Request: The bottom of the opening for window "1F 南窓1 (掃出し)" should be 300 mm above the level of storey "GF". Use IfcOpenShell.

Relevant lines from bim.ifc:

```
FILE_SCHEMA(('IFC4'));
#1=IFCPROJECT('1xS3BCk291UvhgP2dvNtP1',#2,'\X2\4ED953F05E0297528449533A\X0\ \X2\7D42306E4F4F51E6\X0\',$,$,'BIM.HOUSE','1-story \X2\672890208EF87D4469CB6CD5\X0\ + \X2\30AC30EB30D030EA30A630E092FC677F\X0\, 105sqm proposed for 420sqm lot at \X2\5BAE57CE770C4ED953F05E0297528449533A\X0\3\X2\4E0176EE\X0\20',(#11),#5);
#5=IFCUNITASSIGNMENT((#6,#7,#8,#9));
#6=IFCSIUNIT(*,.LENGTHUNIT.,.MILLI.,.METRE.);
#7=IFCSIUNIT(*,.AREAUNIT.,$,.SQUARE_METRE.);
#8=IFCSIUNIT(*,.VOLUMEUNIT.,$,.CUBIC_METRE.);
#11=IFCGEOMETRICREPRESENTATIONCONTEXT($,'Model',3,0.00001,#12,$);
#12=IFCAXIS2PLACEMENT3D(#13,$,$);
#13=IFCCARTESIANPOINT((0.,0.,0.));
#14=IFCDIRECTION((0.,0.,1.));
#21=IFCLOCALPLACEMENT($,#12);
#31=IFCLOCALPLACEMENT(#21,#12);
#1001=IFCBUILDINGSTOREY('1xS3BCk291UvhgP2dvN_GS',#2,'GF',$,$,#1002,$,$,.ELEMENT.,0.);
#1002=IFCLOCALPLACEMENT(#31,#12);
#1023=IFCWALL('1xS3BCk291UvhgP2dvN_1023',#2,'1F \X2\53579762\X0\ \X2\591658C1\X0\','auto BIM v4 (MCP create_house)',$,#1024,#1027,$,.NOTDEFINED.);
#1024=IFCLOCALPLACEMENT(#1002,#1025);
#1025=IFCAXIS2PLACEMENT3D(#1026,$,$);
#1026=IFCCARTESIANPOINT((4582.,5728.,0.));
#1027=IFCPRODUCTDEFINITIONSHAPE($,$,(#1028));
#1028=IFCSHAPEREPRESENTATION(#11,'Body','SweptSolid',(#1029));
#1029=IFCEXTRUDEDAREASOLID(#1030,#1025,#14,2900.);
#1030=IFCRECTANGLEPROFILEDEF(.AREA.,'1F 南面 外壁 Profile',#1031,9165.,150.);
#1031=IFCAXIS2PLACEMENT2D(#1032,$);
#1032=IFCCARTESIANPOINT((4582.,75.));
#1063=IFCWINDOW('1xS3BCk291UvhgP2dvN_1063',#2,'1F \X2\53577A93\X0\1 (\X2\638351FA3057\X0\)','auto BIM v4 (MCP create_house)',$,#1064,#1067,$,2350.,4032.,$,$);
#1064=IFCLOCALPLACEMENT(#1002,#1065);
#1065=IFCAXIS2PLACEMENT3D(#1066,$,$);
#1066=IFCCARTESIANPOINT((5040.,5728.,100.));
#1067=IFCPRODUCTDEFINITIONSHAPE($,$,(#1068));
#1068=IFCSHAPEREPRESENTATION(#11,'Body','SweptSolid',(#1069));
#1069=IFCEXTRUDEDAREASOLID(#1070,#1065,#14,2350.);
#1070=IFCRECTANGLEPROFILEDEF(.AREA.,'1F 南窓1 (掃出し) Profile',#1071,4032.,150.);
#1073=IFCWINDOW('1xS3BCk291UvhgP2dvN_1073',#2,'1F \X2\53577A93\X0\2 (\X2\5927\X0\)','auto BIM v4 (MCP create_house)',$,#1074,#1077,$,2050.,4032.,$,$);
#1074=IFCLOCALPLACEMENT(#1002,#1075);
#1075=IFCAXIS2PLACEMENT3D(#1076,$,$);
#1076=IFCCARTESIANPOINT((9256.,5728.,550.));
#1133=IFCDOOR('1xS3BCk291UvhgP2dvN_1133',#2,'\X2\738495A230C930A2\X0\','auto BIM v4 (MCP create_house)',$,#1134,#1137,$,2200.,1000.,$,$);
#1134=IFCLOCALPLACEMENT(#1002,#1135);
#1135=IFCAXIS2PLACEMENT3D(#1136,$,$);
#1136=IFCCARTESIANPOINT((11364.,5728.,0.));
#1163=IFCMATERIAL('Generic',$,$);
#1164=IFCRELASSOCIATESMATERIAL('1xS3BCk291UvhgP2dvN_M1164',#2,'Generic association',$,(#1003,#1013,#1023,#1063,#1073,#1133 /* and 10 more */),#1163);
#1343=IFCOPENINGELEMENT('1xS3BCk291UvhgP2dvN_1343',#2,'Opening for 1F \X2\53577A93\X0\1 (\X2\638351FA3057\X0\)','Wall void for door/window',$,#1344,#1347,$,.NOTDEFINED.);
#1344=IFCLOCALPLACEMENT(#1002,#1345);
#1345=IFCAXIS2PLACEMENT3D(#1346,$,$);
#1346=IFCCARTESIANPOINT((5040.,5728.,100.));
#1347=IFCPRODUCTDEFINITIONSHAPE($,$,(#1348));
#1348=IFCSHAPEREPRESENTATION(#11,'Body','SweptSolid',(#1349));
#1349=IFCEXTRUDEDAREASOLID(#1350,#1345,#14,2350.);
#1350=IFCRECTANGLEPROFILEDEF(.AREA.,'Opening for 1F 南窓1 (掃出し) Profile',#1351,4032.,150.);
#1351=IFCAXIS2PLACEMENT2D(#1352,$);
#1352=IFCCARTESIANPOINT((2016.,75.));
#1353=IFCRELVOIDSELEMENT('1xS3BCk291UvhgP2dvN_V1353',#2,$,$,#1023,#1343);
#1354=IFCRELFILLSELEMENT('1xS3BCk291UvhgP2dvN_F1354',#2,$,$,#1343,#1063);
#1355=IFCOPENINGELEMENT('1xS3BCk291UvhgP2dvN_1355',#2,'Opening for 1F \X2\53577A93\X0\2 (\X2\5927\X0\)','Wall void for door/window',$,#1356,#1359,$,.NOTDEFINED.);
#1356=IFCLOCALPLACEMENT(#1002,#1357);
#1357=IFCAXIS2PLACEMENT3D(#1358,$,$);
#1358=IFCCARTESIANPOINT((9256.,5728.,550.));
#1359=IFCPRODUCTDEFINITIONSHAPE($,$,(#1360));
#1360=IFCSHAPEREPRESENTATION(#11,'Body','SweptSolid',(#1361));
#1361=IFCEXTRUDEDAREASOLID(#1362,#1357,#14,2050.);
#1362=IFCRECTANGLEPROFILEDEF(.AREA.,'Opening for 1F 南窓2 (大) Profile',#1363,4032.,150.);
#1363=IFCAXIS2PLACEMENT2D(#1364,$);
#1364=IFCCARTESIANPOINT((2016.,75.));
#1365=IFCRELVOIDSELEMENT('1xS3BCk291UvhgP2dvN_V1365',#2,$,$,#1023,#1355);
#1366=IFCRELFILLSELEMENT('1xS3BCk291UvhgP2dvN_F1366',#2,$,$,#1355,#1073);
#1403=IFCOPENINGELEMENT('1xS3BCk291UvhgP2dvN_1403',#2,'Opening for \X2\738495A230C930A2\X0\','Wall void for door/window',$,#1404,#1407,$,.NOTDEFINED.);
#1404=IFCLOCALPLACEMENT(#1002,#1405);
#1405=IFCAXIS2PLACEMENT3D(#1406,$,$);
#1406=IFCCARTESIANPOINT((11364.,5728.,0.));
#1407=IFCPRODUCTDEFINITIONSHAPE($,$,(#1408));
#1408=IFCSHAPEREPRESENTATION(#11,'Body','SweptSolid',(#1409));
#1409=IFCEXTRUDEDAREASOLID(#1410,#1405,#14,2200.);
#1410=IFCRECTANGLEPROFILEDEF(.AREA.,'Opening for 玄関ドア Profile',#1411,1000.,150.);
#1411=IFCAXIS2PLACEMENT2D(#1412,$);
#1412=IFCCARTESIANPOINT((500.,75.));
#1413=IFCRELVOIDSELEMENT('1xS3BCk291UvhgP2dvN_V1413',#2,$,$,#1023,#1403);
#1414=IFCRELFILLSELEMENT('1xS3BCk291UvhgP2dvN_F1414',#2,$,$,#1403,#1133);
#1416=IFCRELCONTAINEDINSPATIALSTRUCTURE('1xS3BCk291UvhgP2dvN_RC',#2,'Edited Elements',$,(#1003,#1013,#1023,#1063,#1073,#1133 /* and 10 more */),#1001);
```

```python
import numpy as np
import ifcopenshell
import ifcopenshell.api.geometry
import ifcopenshell.geom
import ifcopenshell.util.element
import ifcopenshell.util.placement
import ifcopenshell.util.shape
import ifcopenshell.util.unit

model = ifcopenshell.open("bim.ifc")
unit_scale = ifcopenshell.util.unit.calculate_unit_scale(model)

window = model.by_guid("1xS3BCk291UvhgP2dvN_1063")
opening = window.FillsVoids[0].RelatingOpeningElement
storey = ifcopenshell.util.element.get_container(window, ifc_class="IfcBuildingStorey")
level = ifcopenshell.util.placement.get_local_placement(storey.ObjectPlacement)[2, 3]

# The opening's origin need not be at the sill, so measure its lowest point.
shape = ifcopenshell.geom.create_shape(ifcopenshell.geom.settings(), opening)
bottom = ifcopenshell.util.shape.get_shape_bottom_elevation(shape, shape.geometry) / unit_scale
dz = level + 300.0 - bottom

shift = np.array([0.0, 0.0, dz])
# The window is not placed relative to its opening, so move both.
for product in (opening, window):
    matrix = ifcopenshell.util.placement.get_local_placement(product.ObjectPlacement)
    matrix[:3, 3] += shift
    ifcopenshell.api.geometry.edit_object_placement(model, product=product, matrix=matrix, is_si=False)

print(f"moved by {dz * unit_scale:+.3f} m")

model.write("bim-out.ifc")
```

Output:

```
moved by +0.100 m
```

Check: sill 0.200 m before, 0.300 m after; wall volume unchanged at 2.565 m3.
